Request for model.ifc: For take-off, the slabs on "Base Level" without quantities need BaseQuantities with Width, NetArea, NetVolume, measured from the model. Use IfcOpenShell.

First a look at what the model holds.

```python
import ifcopenshell
import ifcopenshell.util.element
import ifcopenshell.util.unit

model = ifcopenshell.open("model.ifc")
print(model.schema)
for unit_type in ("LENGTHUNIT", "AREAUNIT", "VOLUMEUNIT"):
    print(unit_type, ifcopenshell.util.unit.calculate_unit_scale(model, unit_type))
storey = next(s for s in model.by_type("IfcBuildingStorey") if s.Name == "Base Level")
slabs = [e for e in ifcopenshell.util.element.get_decomposition(storey) if e.is_a("IfcSlab")]
for e in sorted(slabs, key=lambda e: e.id()):
    print(e.id(), e.is_a(), e.Name, list(ifcopenshell.util.element.get_psets(e, qtos_only=True)), sep=" | ")
```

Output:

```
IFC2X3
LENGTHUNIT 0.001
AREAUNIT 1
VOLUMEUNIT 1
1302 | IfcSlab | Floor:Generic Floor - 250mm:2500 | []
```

```python
import ifcopenshell
import ifcopenshell.api.pset
import ifcopenshell.geom
import ifcopenshell.util.element
import ifcopenshell.util.shape
import ifcopenshell.util.unit

model = ifcopenshell.open("model.ifc")
unit_scale = ifcopenshell.util.unit.calculate_unit_scale(model)
area_scale = ifcopenshell.util.unit.calculate_unit_scale(model, "AREAUNIT")
volume_scale = ifcopenshell.util.unit.calculate_unit_scale(model, "VOLUMEUNIT")
settings = ifcopenshell.geom.settings()

storey = next(s for s in model.by_type("IfcBuildingStorey") if s.Name == "Base Level")
slabs = [e for e in ifcopenshell.util.element.get_decomposition(storey) if e.is_a("IfcSlab")]

for e in sorted(slabs, key=lambda e: e.id()):
    if ifcopenshell.util.element.get_psets(e, qtos_only=True, should_inherit=False):
        continue
    # Geometry comes back in metres, in the element's own axes.
    shape = ifcopenshell.geom.create_shape(settings, e)
    values = {
        "Width": ifcopenshell.util.shape.get_z(shape.geometry) / unit_scale,
        "NetArea": ifcopenshell.util.shape.get_footprint_area(shape.geometry) / area_scale,
        "NetVolume": ifcopenshell.util.shape.get_volume(shape.geometry) / volume_scale,
    }
    qto = ifcopenshell.api.pset.add_qto(model, product=e, name="BaseQuantities")
    ifcopenshell.api.pset.edit_qto(model, qto=qto, properties=values)
    print(e.id(), {k: round(v, 3) for k, v in values.items()})

model.write("model-out.ifc")
```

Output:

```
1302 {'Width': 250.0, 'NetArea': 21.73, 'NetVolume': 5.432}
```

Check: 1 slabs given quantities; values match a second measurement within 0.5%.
